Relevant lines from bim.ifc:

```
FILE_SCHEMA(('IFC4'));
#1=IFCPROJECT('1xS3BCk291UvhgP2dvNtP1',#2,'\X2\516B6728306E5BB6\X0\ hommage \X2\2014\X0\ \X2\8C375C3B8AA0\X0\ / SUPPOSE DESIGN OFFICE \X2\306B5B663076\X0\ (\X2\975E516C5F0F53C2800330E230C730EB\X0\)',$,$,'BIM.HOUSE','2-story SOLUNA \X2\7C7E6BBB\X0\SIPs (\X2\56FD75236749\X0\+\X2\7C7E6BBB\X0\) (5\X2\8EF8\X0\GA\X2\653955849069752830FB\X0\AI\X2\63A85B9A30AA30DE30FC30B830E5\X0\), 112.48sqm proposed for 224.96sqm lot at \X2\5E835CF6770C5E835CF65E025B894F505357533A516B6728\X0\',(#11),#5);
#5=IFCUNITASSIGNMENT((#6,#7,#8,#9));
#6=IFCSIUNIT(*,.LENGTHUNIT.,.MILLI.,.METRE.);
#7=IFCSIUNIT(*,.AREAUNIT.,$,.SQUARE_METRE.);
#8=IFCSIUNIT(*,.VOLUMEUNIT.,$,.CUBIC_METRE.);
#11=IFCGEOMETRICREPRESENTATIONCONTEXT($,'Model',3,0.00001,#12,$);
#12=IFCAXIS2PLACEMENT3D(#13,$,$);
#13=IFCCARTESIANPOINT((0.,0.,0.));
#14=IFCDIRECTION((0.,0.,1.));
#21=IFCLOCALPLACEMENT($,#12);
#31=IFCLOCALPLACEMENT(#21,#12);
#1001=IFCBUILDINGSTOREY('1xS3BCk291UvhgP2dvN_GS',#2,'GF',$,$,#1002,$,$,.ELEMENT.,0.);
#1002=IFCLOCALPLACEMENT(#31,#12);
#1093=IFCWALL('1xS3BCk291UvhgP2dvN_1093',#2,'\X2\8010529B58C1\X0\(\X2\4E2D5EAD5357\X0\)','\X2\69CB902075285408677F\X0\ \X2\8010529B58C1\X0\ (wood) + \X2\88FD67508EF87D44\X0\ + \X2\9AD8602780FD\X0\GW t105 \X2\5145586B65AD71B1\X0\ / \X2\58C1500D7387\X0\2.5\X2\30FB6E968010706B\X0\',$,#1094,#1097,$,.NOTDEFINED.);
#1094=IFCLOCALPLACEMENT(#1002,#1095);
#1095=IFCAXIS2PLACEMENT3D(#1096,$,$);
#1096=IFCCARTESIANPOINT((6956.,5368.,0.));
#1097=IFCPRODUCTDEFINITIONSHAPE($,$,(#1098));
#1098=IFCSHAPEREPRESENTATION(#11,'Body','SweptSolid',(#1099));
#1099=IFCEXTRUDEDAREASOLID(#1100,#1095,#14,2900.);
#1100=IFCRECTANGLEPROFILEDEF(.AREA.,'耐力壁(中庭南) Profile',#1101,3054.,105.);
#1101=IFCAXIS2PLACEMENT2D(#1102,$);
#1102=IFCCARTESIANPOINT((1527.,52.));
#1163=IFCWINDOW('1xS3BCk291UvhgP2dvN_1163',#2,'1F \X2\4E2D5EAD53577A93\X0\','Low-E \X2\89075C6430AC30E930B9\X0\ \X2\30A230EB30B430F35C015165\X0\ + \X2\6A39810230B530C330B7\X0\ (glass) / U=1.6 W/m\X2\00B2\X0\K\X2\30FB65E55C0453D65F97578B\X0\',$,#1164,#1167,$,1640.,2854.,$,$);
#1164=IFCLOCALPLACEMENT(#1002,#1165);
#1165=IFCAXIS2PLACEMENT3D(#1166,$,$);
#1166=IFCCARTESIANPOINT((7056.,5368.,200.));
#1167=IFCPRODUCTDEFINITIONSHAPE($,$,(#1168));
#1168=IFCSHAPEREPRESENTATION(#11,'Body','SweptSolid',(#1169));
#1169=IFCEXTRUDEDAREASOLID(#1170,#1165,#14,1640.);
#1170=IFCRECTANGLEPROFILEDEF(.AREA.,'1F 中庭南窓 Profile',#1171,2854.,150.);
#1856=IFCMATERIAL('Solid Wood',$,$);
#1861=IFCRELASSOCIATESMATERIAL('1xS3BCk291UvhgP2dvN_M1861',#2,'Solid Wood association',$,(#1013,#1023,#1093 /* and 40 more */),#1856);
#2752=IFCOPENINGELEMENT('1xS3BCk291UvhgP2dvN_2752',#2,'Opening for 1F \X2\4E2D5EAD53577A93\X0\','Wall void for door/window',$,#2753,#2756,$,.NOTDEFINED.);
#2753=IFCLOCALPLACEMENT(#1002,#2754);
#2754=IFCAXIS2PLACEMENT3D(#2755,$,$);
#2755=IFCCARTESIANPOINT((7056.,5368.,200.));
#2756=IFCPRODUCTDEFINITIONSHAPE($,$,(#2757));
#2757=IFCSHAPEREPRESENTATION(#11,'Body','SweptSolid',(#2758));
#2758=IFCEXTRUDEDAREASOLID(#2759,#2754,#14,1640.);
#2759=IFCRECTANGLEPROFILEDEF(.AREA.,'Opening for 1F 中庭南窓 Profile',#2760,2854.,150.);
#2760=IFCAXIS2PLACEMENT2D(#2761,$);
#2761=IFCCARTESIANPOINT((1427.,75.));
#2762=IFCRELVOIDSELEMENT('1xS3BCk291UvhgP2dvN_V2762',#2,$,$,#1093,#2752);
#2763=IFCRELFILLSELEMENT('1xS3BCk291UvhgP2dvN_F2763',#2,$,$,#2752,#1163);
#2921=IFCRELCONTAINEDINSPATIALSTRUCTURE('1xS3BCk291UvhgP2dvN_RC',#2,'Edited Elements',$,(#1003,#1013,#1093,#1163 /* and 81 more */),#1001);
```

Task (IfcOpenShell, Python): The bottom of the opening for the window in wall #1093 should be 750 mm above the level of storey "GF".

```python
import numpy as np
import ifcopenshell
import ifcopenshell.api.geometry
import ifcopenshell.geom
import ifcopenshell.util.element
import ifcopenshell.util.placement
import ifcopenshell.util.shape
import ifcopenshell.util.unit

model = ifcopenshell.open("bim.ifc")
unit_scale = ifcopenshell.util.unit.calculate_unit_scale(model)

window = model.by_id(1163)
opening = window.FillsVoids[0].RelatingOpeningElement
storey = ifcopenshell.util.element.get_container(window, ifc_class="IfcBuildingStorey")
level = ifcopenshell.util.placement.get_local_placement(storey.ObjectPlacement)[2, 3]

# The opening's origin need not be at the sill, so measure its lowest point.
shape = ifcopenshell.geom.create_shape(ifcopenshell.geom.settings(), opening)
bottom = ifcopenshell.util.shape.get_shape_bottom_elevation(shape, shape.geometry) / unit_scale
dz = level + 750.0 - bottom

shift = np.array([0.0, 0.0, dz])
# The window is not placed relative to its opening, so move both.
for product in (opening, window):
    matrix = ifcopenshell.util.placement.get_local_placement(product.ObjectPlacement)
    matrix[:3, 3] += shift
    ifcopenshell.api.geometry.edit_object_placement(model, product=product, matrix=matrix, is_si=False)

print(f"moved by {dz * unit_scale:+.3f} m")

model.write("bim_edited.ifc")
```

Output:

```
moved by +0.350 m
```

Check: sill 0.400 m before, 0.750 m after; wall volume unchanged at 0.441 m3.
